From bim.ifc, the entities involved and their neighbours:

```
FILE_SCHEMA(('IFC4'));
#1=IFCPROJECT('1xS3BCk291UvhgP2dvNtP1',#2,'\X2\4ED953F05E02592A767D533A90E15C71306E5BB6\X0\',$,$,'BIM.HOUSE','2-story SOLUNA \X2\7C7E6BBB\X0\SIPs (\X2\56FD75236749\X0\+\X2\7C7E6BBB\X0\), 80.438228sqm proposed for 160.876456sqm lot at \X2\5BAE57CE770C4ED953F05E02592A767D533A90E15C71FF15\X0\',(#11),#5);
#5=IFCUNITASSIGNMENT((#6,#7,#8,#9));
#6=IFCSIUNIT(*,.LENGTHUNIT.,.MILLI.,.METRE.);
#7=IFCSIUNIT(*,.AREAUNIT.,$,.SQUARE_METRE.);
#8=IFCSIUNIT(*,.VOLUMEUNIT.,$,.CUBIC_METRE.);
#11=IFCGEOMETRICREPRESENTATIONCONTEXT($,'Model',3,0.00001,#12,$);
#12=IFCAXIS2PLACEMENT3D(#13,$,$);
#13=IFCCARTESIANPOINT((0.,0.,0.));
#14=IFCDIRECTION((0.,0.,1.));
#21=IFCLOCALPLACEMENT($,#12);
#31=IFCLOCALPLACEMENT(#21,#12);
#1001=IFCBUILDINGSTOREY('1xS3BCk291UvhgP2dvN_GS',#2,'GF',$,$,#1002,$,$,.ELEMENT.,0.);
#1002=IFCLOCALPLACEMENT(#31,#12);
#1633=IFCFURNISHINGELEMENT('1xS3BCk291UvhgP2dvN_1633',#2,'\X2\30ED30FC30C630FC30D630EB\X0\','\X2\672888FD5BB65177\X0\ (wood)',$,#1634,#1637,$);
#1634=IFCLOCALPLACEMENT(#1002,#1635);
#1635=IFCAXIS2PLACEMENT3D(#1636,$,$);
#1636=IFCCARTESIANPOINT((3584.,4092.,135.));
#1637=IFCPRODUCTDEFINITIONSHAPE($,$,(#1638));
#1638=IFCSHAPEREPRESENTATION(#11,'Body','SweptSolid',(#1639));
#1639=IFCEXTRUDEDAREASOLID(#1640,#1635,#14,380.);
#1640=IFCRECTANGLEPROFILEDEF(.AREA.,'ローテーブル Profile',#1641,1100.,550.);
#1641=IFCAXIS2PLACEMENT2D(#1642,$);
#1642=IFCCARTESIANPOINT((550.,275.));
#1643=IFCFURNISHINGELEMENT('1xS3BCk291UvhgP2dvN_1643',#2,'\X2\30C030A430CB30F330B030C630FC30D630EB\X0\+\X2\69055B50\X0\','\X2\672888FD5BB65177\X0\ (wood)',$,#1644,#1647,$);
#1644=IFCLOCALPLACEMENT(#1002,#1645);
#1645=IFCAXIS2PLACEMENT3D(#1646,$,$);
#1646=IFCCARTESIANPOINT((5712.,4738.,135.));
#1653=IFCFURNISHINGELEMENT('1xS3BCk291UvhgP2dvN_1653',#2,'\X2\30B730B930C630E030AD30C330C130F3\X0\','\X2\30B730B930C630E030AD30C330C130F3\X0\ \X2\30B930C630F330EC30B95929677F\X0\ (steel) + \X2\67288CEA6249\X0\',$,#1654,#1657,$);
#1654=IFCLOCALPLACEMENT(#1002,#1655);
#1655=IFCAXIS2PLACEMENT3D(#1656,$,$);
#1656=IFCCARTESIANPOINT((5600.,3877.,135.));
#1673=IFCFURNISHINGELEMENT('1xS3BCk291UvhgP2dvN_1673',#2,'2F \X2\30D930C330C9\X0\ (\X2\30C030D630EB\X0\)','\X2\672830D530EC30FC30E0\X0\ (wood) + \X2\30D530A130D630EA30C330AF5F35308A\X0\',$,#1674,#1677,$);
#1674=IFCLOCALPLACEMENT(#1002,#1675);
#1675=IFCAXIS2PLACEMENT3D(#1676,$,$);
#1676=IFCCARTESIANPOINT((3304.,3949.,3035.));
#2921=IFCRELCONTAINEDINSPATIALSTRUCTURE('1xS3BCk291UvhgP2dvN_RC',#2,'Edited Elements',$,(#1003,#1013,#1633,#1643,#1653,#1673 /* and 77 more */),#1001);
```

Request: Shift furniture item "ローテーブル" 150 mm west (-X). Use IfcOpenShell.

```python
import ifcopenshell
import ifcopenshell.api.geometry
import ifcopenshell.util.placement
import ifcopenshell.util.unit

model = ifcopenshell.open("bim.ifc")
unit_scale = ifcopenshell.util.unit.calculate_unit_scale(model)

item = model.by_id(1633)
matrix = ifcopenshell.util.placement.get_local_placement(item.ObjectPlacement)
matrix[0, 3] -= 0.15 / unit_scale
ifcopenshell.api.geometry.edit_object_placement(model, product=item, matrix=matrix, is_si=False)

print(ifcopenshell.util.placement.get_local_placement(item.ObjectPlacement).round(3) + 0.0)

model.write("bim-out.ifc")
```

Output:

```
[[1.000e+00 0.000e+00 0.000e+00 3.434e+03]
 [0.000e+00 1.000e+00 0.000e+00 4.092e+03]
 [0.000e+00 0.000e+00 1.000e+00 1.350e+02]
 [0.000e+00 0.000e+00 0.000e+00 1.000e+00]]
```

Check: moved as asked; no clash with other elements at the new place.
